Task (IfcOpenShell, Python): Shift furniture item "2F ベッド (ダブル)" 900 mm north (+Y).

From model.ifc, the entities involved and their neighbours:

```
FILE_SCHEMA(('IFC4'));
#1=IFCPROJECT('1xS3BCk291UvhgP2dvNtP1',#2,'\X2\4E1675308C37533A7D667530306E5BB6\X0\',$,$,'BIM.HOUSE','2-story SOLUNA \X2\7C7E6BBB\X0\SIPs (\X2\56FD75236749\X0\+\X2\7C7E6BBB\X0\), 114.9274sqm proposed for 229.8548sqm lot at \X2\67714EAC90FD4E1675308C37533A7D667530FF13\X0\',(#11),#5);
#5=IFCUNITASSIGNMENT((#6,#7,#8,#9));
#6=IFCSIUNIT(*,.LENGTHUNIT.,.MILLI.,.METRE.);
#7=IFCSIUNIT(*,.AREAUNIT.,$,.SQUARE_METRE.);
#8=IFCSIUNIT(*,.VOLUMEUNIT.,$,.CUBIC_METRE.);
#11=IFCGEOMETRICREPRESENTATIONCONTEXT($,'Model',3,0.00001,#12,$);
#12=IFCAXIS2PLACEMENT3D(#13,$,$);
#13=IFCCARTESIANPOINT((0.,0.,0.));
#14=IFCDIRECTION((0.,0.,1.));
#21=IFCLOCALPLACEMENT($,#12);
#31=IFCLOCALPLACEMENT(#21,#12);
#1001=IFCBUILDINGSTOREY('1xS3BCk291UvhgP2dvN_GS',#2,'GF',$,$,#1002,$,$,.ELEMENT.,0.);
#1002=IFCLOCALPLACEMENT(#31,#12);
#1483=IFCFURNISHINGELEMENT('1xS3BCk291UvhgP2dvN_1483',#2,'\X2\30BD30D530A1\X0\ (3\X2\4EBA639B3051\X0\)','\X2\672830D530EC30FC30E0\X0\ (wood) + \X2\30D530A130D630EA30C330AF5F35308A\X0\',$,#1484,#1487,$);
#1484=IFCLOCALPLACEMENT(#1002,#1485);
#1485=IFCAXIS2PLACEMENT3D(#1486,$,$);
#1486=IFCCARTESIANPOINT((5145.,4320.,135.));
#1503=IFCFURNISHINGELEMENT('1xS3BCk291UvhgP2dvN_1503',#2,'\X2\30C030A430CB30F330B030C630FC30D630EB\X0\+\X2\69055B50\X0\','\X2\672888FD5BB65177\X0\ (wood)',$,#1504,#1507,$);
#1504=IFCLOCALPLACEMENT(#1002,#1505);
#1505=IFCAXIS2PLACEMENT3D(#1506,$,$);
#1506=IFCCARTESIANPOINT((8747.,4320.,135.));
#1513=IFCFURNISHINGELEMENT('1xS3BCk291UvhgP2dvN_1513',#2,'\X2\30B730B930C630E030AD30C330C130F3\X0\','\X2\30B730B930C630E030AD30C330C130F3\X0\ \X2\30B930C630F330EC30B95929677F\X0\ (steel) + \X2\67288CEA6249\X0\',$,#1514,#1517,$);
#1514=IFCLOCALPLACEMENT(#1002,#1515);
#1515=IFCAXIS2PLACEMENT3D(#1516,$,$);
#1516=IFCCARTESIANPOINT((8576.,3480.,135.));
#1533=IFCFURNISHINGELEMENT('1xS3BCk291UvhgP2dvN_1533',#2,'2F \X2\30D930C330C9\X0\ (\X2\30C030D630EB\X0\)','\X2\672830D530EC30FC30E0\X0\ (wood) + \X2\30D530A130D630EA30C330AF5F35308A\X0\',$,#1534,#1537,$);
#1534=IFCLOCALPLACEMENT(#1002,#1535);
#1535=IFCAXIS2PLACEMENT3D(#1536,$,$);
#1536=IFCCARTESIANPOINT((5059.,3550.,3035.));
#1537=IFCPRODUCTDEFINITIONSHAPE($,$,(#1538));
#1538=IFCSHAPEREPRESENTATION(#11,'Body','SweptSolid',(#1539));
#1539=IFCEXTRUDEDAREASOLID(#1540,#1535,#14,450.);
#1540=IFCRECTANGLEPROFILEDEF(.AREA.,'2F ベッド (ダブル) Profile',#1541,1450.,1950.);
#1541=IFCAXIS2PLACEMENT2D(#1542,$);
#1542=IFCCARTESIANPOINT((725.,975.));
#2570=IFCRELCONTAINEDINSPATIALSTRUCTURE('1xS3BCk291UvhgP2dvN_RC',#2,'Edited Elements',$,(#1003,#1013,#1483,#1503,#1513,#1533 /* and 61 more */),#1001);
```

```python
import ifcopenshell
import ifcopenshell.api.geometry
import ifcopenshell.util.placement
import ifcopenshell.util.unit

model = ifcopenshell.open("model.ifc")
unit_scale = ifcopenshell.util.unit.calculate_unit_scale(model)

item = model.by_guid("1xS3BCk291UvhgP2dvN_1533")
matrix = ifcopenshell.util.placement.get_local_placement(item.ObjectPlacement)
matrix[1, 3] += 0.9 / unit_scale
ifcopenshell.api.geometry.edit_object_placement(model, product=item, matrix=matrix, is_si=False)

print(ifcopenshell.util.placement.get_local_placement(item.ObjectPlacement).round(3) + 0.0)

model.write("model-out.ifc")
```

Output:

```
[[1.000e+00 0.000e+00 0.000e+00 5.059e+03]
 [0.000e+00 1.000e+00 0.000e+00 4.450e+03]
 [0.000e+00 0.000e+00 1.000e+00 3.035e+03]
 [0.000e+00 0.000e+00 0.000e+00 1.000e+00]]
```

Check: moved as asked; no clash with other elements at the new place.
